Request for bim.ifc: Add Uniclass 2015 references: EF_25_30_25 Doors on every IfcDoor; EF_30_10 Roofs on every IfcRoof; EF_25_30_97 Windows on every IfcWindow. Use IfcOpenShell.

First a look at what the model holds.

```python
import ifcopenshell

model = ifcopenshell.open("bim.ifc")
print(model.schema)
print("classifications:", [c.Name for c in model.by_type("IfcClassification")])
for ifc_class in ("IfcDoor", "IfcRoof", "IfcStair", "IfcWall", "IfcWindow"):
    print(ifc_class, len(model.by_type(ifc_class)))
```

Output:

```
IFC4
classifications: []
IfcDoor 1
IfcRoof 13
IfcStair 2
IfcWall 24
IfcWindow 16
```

```python
import ifcopenshell
import ifcopenshell.api.classification

model = ifcopenshell.open("bim.ifc")

system = ifcopenshell.api.classification.add_classification(model, classification="Uniclass 2015")

codes = {
    "IfcDoor": ("EF_25_30_25", "Doors"),
    "IfcRoof": ("EF_30_10", "Roofs"),
    "IfcWindow": ("EF_25_30_97", "Windows"),
}
for ifc_class, (code, name) in codes.items():
    products = model.by_type(ifc_class)
    ifcopenshell.api.classification.add_reference(
        model, products=products, classification=system, identification=code, name=name
    )
    print(code, len(products))

model.write("bim_updated.ifc")
```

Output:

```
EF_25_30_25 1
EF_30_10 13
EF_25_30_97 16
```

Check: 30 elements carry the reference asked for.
